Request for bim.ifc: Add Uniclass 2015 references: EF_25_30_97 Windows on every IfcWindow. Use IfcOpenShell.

First a look at what the model holds.

```python
import ifcopenshell

model = ifcopenshell.open("bim.ifc")
print(model.schema)
print("classifications:", [c.Name for c in model.by_type("IfcClassification")])
for ifc_class in ("IfcDoor", "IfcRoof", "IfcStair", "IfcWall", "IfcWindow"):
    print(ifc_class, len(model.by_type(ifc_class)))
```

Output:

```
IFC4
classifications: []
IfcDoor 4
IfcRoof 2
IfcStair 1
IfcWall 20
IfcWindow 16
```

```python
import ifcopenshell
import ifcopenshell.api.classification

model = ifcopenshell.open("bim.ifc")

system = ifcopenshell.api.classification.add_classification(model, classification="Uniclass 2015")

codes = {
    "IfcWindow": ("EF_25_30_97", "Windows"),
}
for ifc_class, (code, name) in codes.items():
    products = model.by_type(ifc_class)
    ifcopenshell.api.classification.add_reference(
        model, products=products, classification=system, identification=code, name=name
    )
    print(code, len(products))

model.write("bim_v2.ifc")
```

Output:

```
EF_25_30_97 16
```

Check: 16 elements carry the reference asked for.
